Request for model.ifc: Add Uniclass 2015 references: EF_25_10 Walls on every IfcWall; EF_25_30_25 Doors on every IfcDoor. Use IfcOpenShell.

First a look at what the model holds.

```python
import ifcopenshell

model = ifcopenshell.open("model.ifc")
print(model.schema)
print("classifications:", [c.Name for c in model.by_type("IfcClassification")])
for ifc_class in ("IfcDoor", "IfcRoof", "IfcStair", "IfcWall", "IfcWindow"):
    print(ifc_class, len(model.by_type(ifc_class)))
```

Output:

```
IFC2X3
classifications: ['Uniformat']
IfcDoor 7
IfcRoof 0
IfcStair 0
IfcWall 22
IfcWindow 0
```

```python
import ifcopenshell
import ifcopenshell.api.classification

model = ifcopenshell.open("model.ifc")

# IFC2X3 requires Source and Edition and has no link from the project to the system.
system = model.create_entity("IfcClassification", Source="NBS", Edition="2015", Name="Uniclass 2015")

codes = {
    "IfcWall": ("EF_25_10", "Walls"),
    "IfcDoor": ("EF_25_30_25", "Doors"),
}
for ifc_class, (code, name) in codes.items():
    products = model.by_type(ifc_class)
    ifcopenshell.api.classification.add_reference(
        model, products=products, classification=system, identification=code, name=name
    )
    print(code, len(products))

model.write("model_v2.ifc")
```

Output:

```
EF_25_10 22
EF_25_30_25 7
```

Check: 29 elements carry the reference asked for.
